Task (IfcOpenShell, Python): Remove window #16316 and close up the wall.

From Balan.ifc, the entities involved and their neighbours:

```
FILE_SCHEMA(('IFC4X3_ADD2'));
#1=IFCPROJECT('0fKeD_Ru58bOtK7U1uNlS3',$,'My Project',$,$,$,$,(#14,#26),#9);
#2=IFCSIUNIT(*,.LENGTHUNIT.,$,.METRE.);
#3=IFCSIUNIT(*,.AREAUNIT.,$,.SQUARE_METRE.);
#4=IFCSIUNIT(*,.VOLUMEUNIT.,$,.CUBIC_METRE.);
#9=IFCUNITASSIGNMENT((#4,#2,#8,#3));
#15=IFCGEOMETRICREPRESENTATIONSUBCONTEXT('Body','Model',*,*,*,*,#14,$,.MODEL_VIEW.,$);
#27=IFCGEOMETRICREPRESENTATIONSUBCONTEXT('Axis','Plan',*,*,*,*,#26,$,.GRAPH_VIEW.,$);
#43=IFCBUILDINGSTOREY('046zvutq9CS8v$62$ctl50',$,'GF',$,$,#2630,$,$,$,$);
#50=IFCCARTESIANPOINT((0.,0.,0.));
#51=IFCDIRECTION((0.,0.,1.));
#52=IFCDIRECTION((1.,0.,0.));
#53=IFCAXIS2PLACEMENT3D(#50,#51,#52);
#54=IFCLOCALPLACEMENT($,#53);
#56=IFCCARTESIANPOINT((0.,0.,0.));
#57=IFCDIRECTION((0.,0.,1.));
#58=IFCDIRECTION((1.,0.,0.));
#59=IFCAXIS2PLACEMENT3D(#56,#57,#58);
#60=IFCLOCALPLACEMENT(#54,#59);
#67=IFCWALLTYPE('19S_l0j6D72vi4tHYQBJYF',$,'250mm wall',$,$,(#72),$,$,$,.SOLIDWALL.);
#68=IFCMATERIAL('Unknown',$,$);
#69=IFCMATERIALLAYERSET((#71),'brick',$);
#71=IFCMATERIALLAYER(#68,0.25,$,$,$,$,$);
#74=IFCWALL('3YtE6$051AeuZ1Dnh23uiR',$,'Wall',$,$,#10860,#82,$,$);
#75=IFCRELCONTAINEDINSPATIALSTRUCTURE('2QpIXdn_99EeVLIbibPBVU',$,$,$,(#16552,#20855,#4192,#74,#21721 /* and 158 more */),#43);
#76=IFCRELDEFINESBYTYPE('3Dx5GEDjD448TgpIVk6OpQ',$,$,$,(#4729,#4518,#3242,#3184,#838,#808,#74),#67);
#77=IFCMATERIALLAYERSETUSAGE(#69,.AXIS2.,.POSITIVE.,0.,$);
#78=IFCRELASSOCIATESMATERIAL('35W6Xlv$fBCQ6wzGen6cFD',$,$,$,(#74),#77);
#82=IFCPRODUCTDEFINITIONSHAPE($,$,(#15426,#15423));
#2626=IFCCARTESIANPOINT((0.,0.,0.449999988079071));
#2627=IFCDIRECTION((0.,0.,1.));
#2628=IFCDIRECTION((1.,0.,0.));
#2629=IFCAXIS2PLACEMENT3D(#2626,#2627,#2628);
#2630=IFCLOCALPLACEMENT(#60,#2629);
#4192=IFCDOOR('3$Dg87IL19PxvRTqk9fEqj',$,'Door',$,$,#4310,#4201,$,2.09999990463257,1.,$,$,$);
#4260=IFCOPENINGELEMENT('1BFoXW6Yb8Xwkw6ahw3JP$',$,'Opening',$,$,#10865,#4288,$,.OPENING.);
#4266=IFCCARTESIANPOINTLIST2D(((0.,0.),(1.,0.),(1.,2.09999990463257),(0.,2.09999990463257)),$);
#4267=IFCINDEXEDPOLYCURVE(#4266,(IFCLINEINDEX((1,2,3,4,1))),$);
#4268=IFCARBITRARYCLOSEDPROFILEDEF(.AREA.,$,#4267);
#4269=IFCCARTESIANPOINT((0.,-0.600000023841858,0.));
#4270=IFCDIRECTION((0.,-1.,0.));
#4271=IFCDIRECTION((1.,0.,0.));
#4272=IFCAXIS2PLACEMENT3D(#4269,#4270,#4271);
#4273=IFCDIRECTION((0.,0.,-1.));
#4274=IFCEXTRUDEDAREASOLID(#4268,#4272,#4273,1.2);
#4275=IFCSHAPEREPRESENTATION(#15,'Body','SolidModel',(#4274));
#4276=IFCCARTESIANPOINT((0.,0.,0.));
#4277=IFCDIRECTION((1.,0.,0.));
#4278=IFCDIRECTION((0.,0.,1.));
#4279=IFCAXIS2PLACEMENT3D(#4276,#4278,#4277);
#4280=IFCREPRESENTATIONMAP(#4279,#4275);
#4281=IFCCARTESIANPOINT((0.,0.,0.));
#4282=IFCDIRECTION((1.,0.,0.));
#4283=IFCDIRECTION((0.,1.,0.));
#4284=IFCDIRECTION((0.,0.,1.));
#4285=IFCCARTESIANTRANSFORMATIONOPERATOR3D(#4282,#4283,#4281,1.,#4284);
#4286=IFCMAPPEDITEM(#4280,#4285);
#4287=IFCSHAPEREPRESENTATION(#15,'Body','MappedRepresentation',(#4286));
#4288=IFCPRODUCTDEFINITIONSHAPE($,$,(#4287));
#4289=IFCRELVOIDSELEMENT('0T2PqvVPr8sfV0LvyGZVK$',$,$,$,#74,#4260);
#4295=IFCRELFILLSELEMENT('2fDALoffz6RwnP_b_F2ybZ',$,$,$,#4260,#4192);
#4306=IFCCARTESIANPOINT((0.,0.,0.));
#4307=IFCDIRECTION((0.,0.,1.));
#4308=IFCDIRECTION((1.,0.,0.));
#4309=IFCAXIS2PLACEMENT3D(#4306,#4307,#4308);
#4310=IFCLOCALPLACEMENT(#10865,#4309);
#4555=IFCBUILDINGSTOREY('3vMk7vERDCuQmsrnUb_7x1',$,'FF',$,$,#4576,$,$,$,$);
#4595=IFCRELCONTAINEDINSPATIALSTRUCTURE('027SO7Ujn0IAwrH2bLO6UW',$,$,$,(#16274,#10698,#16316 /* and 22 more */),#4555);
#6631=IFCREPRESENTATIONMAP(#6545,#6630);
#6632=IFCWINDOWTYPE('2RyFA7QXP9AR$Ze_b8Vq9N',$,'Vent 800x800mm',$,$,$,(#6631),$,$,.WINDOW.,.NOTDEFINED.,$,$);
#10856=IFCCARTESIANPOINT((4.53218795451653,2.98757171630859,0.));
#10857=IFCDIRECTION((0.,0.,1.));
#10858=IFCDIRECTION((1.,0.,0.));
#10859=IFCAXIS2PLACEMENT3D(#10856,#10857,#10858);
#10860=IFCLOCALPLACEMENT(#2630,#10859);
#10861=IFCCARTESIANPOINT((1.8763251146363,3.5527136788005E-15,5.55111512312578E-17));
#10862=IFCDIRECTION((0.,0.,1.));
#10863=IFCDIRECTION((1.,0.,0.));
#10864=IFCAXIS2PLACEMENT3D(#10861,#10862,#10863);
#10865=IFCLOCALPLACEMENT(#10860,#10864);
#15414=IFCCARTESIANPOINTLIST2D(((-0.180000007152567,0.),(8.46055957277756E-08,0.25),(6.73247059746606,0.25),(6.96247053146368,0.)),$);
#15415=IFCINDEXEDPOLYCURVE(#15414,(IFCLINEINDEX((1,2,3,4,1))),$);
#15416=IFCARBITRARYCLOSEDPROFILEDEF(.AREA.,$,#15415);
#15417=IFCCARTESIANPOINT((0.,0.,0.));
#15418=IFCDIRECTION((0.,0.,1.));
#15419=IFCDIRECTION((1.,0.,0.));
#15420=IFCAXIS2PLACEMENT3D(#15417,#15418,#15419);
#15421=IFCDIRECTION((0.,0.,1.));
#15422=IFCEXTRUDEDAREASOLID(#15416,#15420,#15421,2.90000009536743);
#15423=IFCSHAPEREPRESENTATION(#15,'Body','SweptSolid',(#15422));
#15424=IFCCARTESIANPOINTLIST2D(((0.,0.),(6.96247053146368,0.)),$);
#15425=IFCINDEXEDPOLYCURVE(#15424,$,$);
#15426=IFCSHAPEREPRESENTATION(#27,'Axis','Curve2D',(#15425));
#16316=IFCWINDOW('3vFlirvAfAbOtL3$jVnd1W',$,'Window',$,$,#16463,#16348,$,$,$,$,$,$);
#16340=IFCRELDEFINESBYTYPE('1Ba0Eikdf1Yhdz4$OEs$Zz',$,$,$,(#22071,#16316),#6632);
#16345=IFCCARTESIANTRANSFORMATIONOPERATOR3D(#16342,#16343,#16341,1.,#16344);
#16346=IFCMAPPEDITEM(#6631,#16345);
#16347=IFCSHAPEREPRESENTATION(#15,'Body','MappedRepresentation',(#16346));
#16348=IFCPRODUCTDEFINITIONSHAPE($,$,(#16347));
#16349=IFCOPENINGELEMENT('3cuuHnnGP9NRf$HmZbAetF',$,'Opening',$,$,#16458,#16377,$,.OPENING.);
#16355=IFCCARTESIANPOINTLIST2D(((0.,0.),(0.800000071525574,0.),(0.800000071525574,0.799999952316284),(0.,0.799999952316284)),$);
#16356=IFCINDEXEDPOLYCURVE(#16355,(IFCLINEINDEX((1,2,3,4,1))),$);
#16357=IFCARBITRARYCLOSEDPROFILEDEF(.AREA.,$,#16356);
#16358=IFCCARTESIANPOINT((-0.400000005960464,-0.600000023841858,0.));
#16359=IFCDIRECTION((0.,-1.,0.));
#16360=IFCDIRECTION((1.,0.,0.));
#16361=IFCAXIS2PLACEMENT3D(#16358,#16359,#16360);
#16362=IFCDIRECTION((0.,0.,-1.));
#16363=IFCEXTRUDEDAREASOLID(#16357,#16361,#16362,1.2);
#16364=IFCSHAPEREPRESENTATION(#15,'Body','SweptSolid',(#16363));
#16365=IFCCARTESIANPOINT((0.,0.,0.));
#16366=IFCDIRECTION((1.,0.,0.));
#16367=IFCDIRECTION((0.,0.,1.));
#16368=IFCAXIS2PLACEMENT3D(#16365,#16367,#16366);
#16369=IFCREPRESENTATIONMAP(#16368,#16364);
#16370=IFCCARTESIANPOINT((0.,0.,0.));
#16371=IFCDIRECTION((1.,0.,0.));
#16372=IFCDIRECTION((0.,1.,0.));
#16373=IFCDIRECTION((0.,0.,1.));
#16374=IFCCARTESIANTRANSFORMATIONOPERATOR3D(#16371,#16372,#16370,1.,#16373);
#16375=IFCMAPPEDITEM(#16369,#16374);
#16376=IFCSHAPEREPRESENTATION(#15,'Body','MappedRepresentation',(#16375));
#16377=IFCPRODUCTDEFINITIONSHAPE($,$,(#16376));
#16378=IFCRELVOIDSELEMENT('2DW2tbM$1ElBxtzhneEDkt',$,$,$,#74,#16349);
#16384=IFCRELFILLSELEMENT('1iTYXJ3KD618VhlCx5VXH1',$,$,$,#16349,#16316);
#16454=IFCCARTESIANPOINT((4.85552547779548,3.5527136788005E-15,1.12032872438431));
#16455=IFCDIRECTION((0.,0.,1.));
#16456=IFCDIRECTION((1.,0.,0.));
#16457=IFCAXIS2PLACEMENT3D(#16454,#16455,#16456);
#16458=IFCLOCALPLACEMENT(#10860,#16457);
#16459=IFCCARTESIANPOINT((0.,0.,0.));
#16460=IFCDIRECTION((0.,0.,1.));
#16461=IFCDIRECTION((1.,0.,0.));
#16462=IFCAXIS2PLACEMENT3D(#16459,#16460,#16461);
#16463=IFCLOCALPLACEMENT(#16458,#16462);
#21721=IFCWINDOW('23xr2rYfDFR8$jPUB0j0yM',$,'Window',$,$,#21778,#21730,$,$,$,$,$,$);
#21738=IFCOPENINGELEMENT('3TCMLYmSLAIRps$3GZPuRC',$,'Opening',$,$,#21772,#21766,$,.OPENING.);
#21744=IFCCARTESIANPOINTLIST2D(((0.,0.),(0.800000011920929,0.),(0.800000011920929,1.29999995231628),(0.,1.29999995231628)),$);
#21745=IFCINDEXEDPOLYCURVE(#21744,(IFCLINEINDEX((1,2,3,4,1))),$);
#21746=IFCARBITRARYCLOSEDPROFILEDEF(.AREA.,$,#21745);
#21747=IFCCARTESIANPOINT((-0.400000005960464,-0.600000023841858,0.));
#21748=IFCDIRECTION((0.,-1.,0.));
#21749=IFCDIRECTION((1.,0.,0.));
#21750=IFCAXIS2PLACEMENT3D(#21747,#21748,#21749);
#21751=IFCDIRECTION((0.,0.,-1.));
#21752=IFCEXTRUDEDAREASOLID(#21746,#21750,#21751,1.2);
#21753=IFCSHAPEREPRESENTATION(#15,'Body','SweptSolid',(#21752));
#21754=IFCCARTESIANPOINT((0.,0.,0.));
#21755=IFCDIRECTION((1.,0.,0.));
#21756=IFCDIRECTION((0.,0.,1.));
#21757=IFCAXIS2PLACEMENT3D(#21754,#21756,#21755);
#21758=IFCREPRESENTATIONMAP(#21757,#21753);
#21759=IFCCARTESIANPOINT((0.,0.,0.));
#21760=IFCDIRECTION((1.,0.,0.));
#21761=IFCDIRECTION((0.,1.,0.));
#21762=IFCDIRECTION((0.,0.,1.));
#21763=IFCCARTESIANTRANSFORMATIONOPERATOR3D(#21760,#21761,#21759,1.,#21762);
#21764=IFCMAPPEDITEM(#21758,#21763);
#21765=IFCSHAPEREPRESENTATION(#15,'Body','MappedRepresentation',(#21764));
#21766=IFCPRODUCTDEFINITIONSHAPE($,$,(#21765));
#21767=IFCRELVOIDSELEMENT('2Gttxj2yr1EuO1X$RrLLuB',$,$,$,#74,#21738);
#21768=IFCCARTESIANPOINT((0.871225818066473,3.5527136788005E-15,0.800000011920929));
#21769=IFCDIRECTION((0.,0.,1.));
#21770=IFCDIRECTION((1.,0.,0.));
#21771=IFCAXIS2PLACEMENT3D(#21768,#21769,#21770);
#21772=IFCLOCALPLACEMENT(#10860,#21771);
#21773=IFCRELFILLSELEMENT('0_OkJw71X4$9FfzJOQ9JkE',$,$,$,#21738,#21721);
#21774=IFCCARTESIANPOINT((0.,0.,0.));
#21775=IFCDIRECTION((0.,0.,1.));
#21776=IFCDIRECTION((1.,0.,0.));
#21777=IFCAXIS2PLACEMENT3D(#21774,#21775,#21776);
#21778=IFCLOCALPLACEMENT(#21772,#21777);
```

```python
import ifcopenshell
import ifcopenshell.api.feature
import ifcopenshell.api.root
import ifcopenshell.geom
import ifcopenshell.util.shape

model = ifcopenshell.open("Balan.ifc")
settings = ifcopenshell.geom.settings()


def volume(element):
    """Net volume in cubic metres, openings subtracted."""
    shape = ifcopenshell.geom.create_shape(settings, element)
    return ifcopenshell.util.shape.get_volume(shape.geometry)


window = model.by_guid("3vFlirvAfAbOtL3$jVnd1W")
opening = window.FillsVoids[0].RelatingOpeningElement
wall = opening.VoidsElements[0].RelatingBuildingElement
before = volume(wall)

ifcopenshell.api.root.remove_product(model, product=window)
ifcopenshell.api.feature.remove_feature(model, feature=opening)

after = volume(wall)

print(f"wall volume {before:.3f} -> {after:.3f} m3")

model.write("Balan_v2.ifc")
```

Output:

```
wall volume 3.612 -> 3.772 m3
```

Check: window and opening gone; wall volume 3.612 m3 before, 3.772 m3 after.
